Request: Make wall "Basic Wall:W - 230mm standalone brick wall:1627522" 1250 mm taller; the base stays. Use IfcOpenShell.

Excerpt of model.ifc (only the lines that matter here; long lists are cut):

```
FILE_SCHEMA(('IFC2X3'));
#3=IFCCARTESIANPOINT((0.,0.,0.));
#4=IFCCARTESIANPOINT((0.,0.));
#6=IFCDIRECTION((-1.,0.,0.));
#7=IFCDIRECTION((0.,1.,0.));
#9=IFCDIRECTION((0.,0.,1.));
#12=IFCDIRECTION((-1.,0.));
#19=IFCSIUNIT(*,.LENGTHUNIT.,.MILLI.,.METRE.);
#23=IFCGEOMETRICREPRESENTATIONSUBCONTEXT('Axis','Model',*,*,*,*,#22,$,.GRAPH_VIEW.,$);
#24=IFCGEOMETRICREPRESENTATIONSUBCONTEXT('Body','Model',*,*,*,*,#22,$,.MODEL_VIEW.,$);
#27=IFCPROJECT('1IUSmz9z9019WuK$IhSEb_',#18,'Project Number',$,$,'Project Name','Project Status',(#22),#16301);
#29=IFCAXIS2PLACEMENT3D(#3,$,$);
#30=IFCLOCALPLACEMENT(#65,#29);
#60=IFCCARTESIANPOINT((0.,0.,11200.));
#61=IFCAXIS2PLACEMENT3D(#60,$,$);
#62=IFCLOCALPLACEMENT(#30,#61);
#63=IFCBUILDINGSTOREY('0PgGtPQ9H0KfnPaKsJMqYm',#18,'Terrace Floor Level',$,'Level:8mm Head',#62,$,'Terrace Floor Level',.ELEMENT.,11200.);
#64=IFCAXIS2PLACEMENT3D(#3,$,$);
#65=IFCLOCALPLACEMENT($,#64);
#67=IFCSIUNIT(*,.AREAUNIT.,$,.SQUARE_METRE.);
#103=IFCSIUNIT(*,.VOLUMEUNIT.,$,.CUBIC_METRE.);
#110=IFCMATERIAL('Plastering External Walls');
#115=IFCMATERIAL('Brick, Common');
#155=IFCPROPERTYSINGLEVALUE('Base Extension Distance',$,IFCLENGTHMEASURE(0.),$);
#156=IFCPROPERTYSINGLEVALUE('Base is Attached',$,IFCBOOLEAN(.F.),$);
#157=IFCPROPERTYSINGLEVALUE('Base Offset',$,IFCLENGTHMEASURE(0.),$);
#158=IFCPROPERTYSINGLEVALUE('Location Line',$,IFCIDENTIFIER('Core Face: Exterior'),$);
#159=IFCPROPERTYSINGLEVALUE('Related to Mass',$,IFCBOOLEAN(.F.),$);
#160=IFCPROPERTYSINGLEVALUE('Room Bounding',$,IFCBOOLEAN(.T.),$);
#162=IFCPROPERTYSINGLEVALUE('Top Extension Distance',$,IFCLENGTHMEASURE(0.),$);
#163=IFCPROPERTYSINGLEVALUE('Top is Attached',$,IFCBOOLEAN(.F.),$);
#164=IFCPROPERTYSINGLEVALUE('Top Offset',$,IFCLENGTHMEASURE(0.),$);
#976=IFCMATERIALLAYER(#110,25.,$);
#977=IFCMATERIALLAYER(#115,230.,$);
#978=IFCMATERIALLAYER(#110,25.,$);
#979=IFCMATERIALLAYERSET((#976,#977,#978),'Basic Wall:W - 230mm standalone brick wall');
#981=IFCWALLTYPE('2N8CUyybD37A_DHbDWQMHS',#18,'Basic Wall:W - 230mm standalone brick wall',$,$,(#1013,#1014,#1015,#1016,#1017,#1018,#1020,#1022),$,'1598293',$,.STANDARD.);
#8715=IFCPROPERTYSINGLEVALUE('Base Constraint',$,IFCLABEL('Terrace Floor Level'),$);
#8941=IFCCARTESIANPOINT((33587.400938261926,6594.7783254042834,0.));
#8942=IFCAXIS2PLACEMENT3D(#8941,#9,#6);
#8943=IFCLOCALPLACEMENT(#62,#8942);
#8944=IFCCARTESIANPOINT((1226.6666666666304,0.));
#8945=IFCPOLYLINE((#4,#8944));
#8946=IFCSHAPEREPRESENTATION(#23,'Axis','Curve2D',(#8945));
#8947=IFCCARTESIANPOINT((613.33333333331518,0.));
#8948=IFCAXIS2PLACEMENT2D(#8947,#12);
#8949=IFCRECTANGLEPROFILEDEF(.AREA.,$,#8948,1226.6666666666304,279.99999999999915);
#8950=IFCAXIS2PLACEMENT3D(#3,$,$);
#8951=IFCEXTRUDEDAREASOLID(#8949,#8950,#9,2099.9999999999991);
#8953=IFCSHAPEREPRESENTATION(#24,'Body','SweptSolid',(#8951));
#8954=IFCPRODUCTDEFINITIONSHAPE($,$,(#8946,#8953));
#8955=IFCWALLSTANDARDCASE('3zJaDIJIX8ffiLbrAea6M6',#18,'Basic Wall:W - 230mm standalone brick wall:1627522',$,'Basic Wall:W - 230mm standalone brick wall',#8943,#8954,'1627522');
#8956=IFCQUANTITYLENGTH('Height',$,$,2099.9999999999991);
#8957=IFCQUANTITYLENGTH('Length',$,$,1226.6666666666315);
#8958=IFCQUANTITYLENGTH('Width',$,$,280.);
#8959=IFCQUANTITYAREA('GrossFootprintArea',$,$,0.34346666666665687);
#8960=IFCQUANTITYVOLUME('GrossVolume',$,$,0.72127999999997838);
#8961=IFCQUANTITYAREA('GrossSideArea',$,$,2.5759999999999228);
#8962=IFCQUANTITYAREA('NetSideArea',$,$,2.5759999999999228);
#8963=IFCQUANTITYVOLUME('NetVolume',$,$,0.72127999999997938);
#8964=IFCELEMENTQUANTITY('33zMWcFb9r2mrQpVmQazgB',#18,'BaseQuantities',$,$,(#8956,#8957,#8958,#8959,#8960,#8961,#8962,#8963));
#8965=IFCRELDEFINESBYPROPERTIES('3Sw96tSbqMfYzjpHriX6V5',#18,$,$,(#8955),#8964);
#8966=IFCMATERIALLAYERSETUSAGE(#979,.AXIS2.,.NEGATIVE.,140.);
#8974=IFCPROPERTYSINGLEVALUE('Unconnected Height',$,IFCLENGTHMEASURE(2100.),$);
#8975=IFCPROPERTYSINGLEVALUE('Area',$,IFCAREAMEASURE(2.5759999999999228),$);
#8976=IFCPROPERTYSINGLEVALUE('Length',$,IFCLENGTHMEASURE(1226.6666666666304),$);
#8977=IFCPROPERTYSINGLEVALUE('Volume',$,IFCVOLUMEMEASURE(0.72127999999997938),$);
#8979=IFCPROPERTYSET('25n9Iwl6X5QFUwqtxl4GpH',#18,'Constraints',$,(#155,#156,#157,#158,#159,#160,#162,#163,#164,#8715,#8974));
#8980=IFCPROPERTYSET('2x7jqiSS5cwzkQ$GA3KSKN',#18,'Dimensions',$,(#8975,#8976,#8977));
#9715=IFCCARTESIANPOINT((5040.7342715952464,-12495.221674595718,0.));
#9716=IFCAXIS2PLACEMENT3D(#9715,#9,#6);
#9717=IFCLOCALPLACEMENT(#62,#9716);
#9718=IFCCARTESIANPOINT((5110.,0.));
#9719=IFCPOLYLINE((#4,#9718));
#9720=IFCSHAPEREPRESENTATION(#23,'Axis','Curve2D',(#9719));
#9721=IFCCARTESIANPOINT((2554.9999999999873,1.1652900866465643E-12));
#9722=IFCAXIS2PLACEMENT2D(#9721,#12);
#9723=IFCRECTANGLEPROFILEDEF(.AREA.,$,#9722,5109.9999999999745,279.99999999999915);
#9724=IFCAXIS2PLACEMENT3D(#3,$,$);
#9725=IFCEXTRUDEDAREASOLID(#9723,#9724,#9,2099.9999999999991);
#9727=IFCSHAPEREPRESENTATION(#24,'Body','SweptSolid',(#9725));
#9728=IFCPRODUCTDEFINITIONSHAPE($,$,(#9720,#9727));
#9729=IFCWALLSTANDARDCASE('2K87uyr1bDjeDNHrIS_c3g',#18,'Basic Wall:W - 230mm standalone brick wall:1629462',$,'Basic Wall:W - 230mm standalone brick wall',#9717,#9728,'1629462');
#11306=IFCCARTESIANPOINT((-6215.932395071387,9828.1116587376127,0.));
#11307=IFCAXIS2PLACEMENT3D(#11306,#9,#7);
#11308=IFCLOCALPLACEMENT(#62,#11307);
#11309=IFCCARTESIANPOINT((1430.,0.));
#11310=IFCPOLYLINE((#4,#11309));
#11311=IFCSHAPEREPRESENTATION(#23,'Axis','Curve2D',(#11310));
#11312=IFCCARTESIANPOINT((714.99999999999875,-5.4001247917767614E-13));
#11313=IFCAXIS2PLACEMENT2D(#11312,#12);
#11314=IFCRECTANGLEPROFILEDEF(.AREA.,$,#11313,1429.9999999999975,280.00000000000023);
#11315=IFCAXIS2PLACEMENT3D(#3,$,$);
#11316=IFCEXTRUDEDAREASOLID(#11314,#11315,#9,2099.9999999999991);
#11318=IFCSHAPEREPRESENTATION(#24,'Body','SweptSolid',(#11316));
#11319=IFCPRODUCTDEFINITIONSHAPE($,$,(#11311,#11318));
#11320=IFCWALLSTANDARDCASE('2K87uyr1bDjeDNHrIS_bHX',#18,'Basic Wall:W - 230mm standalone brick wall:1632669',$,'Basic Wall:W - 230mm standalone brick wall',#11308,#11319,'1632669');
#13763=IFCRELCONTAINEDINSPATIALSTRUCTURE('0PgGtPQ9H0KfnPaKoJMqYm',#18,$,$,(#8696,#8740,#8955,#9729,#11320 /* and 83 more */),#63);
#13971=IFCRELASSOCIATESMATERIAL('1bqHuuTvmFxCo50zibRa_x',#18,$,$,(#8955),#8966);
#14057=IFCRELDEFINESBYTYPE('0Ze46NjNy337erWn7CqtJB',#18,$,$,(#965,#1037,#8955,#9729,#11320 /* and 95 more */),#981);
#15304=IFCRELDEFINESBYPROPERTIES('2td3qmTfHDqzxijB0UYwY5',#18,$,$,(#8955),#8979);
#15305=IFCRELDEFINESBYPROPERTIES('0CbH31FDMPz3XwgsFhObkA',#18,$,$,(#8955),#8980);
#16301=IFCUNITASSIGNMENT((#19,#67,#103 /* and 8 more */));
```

```python
import ifcopenshell
import ifcopenshell.api.pset
import ifcopenshell.geom
import ifcopenshell.util.element
import ifcopenshell.util.representation
import ifcopenshell.util.shape
import ifcopenshell.util.unit

model = ifcopenshell.open("model.ifc")
unit_scale = ifcopenshell.util.unit.calculate_unit_scale(model)
area_scale = ifcopenshell.util.unit.calculate_unit_scale(model, "AREAUNIT")
volume_scale = ifcopenshell.util.unit.calculate_unit_scale(model, "VOLUMEUNIT")
settings = ifcopenshell.geom.settings()


def volume(element):
    """Net volume in cubic metres, openings subtracted."""
    shape = ifcopenshell.geom.create_shape(settings, element)
    return ifcopenshell.util.shape.get_volume(shape.geometry)


wall = model.by_guid("3zJaDIJIX8ffiLbrAea6M6")
before = volume(wall)

body = ifcopenshell.util.representation.get_representation(wall, "Model", "Body")
solid = body.Items[0]
old_height = solid.Depth
solid.Depth += 1.25 / unit_scale
after = volume(wall)
thickness = 0.28  # wall thickness in metres

# Update the stored height, areas and volumes.
qto = model.by_id(ifcopenshell.util.element.get_pset(wall, "BaseQuantities", should_inherit=False)["id"])
ifcopenshell.api.pset.edit_qto(model, qto=qto, properties={
    "Height": solid.Depth,
    "GrossVolume": ifcopenshell.util.element.get_pset(wall, "BaseQuantities", "GrossVolume") * solid.Depth / old_height,
    "GrossSideArea": ifcopenshell.util.element.get_pset(wall, "BaseQuantities", "GrossSideArea") * solid.Depth / old_height,
    "NetSideArea": after / thickness / area_scale,
    "NetVolume": after / volume_scale,
})
pset = model.by_id(ifcopenshell.util.element.get_pset(wall, "Constraints", should_inherit=False)["id"])
ifcopenshell.api.pset.edit_pset(model, pset=pset, properties={
    "Unconnected Height": model.create_entity("IfcLengthMeasure", solid.Depth),
})
pset = model.by_id(ifcopenshell.util.element.get_pset(wall, "Dimensions", should_inherit=False)["id"])
ifcopenshell.api.pset.edit_pset(model, pset=pset, properties={
    "Area": model.create_entity("IfcAreaMeasure", after / thickness / area_scale),
    "Volume": model.create_entity("IfcVolumeMeasure", after / volume_scale),
})

print(f"height {old_height:g} -> {solid.Depth:g}, volume {before:.3f} -> {after:.3f} m3")

model.write("model_edited.ifc")
```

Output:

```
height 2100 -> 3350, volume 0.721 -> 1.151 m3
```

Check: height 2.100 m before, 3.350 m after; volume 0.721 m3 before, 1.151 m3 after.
